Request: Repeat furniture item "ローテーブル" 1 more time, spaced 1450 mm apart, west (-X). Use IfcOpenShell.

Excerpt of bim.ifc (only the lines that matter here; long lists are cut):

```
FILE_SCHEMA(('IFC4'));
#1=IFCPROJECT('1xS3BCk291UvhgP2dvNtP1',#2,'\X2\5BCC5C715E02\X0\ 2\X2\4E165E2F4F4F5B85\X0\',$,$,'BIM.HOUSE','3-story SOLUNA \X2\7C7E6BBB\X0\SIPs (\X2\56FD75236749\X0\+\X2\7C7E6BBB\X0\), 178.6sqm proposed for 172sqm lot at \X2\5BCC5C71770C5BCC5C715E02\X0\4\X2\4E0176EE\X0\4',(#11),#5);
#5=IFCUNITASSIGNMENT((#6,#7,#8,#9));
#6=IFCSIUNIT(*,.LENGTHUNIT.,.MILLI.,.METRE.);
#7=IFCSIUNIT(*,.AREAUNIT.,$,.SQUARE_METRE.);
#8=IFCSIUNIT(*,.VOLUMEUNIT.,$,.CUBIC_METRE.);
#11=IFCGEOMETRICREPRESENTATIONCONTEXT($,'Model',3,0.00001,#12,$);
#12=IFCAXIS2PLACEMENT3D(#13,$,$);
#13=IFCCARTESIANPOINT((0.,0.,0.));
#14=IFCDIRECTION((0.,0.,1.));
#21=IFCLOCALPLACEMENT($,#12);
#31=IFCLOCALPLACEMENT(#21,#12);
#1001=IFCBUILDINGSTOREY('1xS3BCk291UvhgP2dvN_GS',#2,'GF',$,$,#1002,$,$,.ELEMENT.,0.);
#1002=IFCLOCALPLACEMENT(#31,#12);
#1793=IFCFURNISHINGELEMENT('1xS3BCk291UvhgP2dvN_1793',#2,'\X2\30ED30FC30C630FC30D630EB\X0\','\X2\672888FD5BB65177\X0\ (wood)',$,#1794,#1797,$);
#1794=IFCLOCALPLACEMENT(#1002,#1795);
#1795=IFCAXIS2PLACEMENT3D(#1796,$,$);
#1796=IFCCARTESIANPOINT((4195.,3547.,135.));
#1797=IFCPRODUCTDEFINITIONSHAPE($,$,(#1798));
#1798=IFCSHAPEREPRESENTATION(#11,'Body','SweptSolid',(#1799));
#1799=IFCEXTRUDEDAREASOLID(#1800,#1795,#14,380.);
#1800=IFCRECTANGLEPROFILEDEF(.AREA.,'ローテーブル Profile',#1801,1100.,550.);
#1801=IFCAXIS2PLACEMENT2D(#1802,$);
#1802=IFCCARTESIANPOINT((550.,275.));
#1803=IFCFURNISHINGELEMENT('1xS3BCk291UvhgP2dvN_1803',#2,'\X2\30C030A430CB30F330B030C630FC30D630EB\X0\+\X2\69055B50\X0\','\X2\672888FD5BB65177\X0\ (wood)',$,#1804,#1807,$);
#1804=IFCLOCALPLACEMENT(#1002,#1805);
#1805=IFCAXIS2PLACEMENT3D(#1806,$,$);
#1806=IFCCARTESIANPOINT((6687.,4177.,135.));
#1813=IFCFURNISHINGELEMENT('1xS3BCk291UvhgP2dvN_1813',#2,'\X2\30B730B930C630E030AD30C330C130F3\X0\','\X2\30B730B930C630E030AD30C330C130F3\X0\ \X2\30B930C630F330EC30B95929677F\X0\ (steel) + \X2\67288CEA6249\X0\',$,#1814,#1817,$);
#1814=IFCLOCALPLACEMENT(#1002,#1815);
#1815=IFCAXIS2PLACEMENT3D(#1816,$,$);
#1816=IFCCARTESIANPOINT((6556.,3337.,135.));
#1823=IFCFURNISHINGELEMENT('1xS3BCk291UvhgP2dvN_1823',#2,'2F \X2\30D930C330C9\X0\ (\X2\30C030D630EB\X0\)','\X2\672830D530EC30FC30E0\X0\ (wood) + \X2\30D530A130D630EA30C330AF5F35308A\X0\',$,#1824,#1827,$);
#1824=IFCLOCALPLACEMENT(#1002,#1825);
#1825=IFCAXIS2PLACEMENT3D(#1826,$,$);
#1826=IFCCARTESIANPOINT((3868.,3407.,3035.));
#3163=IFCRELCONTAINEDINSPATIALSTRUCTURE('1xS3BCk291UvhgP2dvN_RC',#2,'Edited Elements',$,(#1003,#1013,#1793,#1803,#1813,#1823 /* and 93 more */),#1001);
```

```python
import numpy as np
import ifcopenshell
import ifcopenshell.api.geometry
import ifcopenshell.api.root
import ifcopenshell.util.element
import ifcopenshell.util.placement
import ifcopenshell.util.unit

model = ifcopenshell.open("bim.ifc")
unit_scale = ifcopenshell.util.unit.calculate_unit_scale(model)


def reuse_history(source, copy):
    """copy_class also copies each property set's owner history, people and application; keep the originals."""
    for rel in copy.IsDefinedBy:
        if rel.is_a("IfcRelDefinesByProperties") and (history := rel.RelatingPropertyDefinition.OwnerHistory):
            rel.RelatingPropertyDefinition.OwnerHistory = source.OwnerHistory
            ifcopenshell.util.element.remove_deep2(model, history)


source = model.by_id(1793)
base = ifcopenshell.util.placement.get_local_placement(source.ObjectPlacement)
step = np.array([-1.0, 0.0, 0.0]) * 1.45 / unit_scale

for i in range(1, 2):
    copy = ifcopenshell.api.root.copy_class(model, product=source)
    copy.Representation = ifcopenshell.util.element.copy_deep(
        model, source.Representation, exclude=["IfcGeometricRepresentationContext", "IfcRepresentationMap"]
    )
    reuse_history(source, copy)
    matrix = base.copy()
    matrix[:3, 3] += i * step
    print("added at", matrix[:3, 3].round(3) + 0.0)
    ifcopenshell.api.geometry.edit_object_placement(model, product=copy, matrix=matrix, is_si=False)

model.write("bim-out.ifc")
```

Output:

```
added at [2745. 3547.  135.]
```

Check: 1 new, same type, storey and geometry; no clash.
